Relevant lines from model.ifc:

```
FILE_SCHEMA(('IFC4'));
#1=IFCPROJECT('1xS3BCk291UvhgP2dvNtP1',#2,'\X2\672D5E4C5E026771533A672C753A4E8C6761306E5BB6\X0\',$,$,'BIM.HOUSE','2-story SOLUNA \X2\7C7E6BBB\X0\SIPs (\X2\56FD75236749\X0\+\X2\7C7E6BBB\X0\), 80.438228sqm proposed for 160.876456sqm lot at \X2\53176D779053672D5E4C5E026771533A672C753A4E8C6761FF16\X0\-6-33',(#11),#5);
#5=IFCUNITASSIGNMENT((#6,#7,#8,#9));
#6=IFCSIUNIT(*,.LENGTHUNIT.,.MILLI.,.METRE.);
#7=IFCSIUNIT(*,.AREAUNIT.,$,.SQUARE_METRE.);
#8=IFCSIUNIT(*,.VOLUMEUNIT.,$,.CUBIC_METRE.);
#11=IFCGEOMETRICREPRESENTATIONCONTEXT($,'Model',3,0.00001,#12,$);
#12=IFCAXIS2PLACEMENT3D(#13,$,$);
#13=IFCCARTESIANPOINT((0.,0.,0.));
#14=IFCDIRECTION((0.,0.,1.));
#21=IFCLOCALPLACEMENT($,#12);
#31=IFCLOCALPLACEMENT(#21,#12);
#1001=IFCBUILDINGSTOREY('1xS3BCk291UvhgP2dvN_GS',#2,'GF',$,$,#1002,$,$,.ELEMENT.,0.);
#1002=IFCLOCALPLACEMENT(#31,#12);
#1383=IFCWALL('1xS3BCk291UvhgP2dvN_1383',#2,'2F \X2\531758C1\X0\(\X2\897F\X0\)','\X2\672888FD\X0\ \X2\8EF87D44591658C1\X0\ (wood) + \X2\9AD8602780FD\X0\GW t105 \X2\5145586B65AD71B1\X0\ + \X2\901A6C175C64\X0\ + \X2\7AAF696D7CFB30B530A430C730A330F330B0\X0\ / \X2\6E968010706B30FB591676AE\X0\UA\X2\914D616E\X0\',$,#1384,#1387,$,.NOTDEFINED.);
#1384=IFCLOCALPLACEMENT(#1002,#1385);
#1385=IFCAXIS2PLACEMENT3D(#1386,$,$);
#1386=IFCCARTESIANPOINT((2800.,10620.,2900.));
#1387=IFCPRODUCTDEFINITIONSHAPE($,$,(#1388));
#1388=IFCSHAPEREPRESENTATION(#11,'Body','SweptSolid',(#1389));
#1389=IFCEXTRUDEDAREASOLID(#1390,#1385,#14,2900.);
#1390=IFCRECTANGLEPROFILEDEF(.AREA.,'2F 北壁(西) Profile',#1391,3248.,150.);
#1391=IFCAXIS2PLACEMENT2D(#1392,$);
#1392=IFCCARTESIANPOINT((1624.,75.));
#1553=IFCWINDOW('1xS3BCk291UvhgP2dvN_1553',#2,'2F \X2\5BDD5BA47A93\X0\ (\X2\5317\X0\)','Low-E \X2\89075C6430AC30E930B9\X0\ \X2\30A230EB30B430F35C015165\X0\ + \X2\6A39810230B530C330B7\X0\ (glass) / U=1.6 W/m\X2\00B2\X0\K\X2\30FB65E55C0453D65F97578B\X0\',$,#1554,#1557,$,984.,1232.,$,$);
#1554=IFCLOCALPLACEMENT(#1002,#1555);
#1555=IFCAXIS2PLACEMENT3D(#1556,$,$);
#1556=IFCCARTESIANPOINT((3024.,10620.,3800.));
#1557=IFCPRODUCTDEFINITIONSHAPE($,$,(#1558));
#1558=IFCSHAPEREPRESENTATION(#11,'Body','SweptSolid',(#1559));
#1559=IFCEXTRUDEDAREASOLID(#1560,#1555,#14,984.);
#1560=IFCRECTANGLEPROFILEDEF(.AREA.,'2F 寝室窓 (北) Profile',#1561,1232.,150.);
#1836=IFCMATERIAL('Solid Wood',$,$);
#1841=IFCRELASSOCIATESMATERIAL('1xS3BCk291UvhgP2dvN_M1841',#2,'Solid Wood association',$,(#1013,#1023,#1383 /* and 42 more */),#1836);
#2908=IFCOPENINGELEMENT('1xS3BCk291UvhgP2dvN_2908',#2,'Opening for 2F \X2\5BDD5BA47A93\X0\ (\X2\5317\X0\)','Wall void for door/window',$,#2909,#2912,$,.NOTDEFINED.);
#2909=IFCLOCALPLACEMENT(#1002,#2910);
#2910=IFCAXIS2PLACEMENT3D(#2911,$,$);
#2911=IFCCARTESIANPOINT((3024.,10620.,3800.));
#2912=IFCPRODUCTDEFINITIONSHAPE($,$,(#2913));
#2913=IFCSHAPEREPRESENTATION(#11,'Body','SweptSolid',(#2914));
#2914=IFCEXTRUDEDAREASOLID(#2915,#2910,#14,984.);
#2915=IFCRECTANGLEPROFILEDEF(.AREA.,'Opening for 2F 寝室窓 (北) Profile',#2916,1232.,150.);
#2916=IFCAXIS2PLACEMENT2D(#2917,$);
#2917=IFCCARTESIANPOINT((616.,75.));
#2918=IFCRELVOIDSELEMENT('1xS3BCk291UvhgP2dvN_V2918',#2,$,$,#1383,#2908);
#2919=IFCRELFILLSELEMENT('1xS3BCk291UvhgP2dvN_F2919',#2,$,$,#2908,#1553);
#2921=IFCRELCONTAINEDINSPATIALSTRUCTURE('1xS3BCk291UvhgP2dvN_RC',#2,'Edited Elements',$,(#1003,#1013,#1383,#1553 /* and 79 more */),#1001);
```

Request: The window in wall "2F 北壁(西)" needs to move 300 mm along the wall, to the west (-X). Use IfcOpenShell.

```python
import ifcopenshell
import ifcopenshell.api.geometry
import ifcopenshell.util.placement
import ifcopenshell.util.unit

model = ifcopenshell.open("model.ifc")
unit_scale = ifcopenshell.util.unit.calculate_unit_scale(model)

window = model.by_id(1553)
opening = window.FillsVoids[0].RelatingOpeningElement
wall = opening.VoidsElements[0].RelatingBuildingElement

wall_matrix = ifcopenshell.util.placement.get_local_placement(wall.ObjectPlacement)
shift = wall_matrix[:3, 0] * -0.3 / unit_scale
before = ifcopenshell.util.placement.get_local_placement(window.ObjectPlacement)[:3, 3].copy()

# The window is not placed relative to its opening, so move both.
for product in (opening, window):
    matrix = ifcopenshell.util.placement.get_local_placement(product.ObjectPlacement)
    matrix[:3, 3] += shift
    ifcopenshell.api.geometry.edit_object_placement(model, product=product, matrix=matrix, is_si=False)

after = ifcopenshell.util.placement.get_local_placement(window.ObjectPlacement)[:3, 3]
print("window moved by", (after - before).round(3) + 0.0)

model.write("model-out.ifc")
```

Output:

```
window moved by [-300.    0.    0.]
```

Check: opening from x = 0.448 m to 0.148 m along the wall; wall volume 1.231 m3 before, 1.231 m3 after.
